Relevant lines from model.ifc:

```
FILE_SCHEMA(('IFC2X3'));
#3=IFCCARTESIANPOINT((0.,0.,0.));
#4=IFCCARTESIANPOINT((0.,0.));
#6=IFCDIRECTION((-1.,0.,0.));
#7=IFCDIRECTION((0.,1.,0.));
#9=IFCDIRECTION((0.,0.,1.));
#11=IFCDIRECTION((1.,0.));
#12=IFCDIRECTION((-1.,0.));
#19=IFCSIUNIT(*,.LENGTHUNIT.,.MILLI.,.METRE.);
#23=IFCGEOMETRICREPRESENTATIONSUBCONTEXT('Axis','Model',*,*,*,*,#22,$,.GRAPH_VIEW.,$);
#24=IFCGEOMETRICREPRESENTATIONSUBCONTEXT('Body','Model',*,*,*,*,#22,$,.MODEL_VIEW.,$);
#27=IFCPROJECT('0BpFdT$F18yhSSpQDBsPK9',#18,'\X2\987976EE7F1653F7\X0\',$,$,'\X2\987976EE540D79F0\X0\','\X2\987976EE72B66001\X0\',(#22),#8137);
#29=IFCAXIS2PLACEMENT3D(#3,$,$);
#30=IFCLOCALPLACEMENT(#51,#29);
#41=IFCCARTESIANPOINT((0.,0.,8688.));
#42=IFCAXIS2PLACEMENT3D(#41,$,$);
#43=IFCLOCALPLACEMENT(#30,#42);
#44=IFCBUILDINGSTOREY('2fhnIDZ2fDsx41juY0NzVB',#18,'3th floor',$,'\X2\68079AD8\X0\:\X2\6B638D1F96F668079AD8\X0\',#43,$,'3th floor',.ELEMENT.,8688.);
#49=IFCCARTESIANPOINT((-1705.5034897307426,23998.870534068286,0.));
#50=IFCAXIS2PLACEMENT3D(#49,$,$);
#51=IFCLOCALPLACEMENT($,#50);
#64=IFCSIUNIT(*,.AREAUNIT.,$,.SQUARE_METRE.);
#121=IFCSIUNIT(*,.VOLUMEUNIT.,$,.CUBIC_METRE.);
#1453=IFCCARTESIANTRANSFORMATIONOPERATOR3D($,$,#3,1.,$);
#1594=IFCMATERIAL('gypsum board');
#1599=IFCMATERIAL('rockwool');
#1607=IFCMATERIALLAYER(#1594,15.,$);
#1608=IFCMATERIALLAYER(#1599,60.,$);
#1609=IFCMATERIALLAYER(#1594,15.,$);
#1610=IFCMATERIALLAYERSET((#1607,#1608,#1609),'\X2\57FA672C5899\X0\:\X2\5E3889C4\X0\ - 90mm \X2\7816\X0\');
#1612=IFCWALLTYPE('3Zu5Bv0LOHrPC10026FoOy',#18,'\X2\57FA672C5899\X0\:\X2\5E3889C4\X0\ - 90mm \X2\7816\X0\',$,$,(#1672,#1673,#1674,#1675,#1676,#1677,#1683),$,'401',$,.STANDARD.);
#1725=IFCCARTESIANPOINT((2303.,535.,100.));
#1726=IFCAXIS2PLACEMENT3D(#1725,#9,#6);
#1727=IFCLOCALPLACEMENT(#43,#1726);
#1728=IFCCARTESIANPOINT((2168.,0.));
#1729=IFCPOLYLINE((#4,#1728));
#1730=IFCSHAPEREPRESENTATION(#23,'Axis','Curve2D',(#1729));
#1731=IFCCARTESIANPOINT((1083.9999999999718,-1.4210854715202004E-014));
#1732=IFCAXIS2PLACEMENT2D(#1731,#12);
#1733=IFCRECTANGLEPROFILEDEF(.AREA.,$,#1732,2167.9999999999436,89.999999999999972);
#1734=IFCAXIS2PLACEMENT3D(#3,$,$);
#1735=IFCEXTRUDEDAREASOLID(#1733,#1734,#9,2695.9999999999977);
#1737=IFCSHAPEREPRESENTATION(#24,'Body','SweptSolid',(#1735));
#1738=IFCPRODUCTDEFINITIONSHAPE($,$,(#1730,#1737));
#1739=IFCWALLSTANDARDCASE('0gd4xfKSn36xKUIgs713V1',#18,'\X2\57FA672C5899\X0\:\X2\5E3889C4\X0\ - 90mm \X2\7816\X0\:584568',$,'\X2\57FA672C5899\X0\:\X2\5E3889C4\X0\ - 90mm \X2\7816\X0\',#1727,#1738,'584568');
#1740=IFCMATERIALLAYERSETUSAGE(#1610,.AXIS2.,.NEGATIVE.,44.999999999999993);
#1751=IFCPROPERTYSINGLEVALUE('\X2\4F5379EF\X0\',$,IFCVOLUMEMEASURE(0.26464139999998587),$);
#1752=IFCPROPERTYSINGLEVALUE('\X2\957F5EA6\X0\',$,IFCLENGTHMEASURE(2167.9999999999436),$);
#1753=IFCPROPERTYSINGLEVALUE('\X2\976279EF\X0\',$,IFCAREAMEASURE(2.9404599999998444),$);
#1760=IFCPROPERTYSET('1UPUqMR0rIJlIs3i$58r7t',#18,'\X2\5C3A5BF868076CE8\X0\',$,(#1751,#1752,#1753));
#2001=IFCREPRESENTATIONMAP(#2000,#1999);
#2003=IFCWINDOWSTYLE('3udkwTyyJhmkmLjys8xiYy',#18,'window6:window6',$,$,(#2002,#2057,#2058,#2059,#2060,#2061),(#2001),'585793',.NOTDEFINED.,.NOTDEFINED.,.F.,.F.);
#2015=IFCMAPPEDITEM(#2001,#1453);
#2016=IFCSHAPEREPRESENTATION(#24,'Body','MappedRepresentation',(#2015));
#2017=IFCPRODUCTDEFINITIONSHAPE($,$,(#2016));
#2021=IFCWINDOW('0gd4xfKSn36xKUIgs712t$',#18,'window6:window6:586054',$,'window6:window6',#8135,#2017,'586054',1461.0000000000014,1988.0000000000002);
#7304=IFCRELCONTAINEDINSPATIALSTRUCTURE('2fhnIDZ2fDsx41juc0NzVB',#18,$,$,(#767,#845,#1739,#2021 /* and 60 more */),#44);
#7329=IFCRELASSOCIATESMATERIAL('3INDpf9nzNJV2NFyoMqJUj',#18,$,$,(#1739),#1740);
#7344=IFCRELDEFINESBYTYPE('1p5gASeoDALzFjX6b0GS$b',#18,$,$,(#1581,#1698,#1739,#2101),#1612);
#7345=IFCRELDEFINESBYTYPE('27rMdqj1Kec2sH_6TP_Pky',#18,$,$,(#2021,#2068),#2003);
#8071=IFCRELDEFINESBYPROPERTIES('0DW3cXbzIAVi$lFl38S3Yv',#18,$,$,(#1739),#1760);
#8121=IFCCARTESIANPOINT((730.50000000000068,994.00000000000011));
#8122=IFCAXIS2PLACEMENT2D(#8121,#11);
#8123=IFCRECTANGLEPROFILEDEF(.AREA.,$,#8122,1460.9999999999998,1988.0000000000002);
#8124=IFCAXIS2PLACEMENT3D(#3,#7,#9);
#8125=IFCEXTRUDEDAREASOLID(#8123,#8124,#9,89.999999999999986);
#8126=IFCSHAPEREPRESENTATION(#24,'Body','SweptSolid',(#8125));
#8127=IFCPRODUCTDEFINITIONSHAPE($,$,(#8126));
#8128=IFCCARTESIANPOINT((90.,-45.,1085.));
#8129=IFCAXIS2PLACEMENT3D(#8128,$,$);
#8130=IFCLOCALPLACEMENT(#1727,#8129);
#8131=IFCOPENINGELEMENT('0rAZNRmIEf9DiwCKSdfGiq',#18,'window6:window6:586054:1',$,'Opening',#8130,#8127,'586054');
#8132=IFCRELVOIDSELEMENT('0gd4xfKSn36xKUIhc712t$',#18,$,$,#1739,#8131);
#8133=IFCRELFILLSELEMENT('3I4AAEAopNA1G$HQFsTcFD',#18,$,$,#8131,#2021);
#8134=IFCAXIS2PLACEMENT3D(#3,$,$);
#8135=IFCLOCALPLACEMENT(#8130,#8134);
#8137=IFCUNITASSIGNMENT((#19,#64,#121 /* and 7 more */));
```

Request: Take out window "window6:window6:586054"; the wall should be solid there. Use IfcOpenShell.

```python
import ifcopenshell
import ifcopenshell.api.feature
import ifcopenshell.api.pset
import ifcopenshell.api.root
import ifcopenshell.geom
import ifcopenshell.util.element
import ifcopenshell.util.shape
import ifcopenshell.util.unit

model = ifcopenshell.open("model.ifc")
area_scale = ifcopenshell.util.unit.calculate_unit_scale(model, "AREAUNIT")
volume_scale = ifcopenshell.util.unit.calculate_unit_scale(model, "VOLUMEUNIT")
settings = ifcopenshell.geom.settings()


def volume(element):
    """Net volume in cubic metres, openings subtracted."""
    shape = ifcopenshell.geom.create_shape(settings, element)
    return ifcopenshell.util.shape.get_volume(shape.geometry)


window = model.by_guid("0gd4xfKSn36xKUIgs712t$")
opening = window.FillsVoids[0].RelatingOpeningElement
wall = opening.VoidsElements[0].RelatingBuildingElement
before = volume(wall)

ifcopenshell.api.root.remove_product(model, product=window)
ifcopenshell.api.feature.remove_feature(model, feature=opening)

after = volume(wall)
thickness = 0.09  # wall thickness in metres

# Update the wall's stored quantities.
pset = model.by_id(ifcopenshell.util.element.get_pset(wall, "尺寸标注", should_inherit=False)["id"])
ifcopenshell.api.pset.edit_pset(model, pset=pset, properties={
    "体积": model.create_entity("IfcVolumeMeasure", after / volume_scale),
    "面积": model.create_entity("IfcAreaMeasure", after / thickness / area_scale),
})

print(f"wall volume {before:.3f} -> {after:.3f} m3")

model.write("model_rev.ifc")
```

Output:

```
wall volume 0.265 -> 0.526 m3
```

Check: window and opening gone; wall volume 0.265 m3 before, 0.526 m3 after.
